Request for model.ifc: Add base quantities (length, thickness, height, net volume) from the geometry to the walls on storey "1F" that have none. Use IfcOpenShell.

First a look at what the model holds.

```python
import ifcopenshell
import ifcopenshell.util.element
import ifcopenshell.util.unit

model = ifcopenshell.open("model.ifc")
print(model.schema)
for unit_type in ("LENGTHUNIT", "AREAUNIT", "VOLUMEUNIT"):
    print(unit_type, ifcopenshell.util.unit.calculate_unit_scale(model, unit_type))
storey = next(s for s in model.by_type("IfcBuildingStorey") if s.Name == "1F")
walls = [e for e in ifcopenshell.util.element.get_decomposition(storey) if e.is_a("IfcWall")]
for e in sorted(walls, key=lambda e: e.id()):
    print(e.id(), e.is_a(), e.Name, list(ifcopenshell.util.element.get_psets(e, qtos_only=True)), sep=" | ")
```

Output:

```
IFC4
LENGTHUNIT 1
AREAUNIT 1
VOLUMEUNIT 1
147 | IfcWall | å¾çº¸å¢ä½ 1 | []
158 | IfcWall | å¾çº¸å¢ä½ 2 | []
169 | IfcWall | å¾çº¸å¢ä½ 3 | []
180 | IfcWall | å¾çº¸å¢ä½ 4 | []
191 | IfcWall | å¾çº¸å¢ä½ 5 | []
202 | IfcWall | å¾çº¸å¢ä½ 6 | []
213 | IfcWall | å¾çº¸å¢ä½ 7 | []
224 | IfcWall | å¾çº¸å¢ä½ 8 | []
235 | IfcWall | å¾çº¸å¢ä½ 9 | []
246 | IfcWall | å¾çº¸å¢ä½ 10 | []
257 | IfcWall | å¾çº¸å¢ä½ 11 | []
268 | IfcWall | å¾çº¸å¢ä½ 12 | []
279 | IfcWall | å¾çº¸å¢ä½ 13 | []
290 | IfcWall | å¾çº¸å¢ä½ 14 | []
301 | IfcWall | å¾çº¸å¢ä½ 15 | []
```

```python
import ifcopenshell
import ifcopenshell.api.pset
import ifcopenshell.geom
import ifcopenshell.util.element
import ifcopenshell.util.shape
import ifcopenshell.util.unit

model = ifcopenshell.open("model.ifc")
unit_scale = ifcopenshell.util.unit.calculate_unit_scale(model)
volume_scale = ifcopenshell.util.unit.calculate_unit_scale(model, "VOLUMEUNIT")
settings = ifcopenshell.geom.settings()

storey = next(s for s in model.by_type("IfcBuildingStorey") if s.Name == "1F")
walls = [e for e in ifcopenshell.util.element.get_decomposition(storey) if e.is_a("IfcWall")]

for e in sorted(walls, key=lambda e: e.id()):
    if ifcopenshell.util.element.get_psets(e, qtos_only=True, should_inherit=False):
        continue
    # Geometry comes back in metres, in the element's own axes.
    shape = ifcopenshell.geom.create_shape(settings, e)
    values = {
        "Length": ifcopenshell.util.shape.get_x(shape.geometry) / unit_scale,
        "Width": ifcopenshell.util.shape.get_y(shape.geometry) / unit_scale,
        "Height": ifcopenshell.util.shape.get_z(shape.geometry) / unit_scale,
        "NetVolume": ifcopenshell.util.shape.get_volume(shape.geometry) / volume_scale,
    }
    qto = ifcopenshell.api.pset.add_qto(model, product=e, name="Qto_WallBaseQuantities")
    ifcopenshell.api.pset.edit_qto(model, qto=qto, properties=values)
    print(e.id(), {k: round(v, 3) for k, v in values.items()})

model.write("model_updated.ifc")
```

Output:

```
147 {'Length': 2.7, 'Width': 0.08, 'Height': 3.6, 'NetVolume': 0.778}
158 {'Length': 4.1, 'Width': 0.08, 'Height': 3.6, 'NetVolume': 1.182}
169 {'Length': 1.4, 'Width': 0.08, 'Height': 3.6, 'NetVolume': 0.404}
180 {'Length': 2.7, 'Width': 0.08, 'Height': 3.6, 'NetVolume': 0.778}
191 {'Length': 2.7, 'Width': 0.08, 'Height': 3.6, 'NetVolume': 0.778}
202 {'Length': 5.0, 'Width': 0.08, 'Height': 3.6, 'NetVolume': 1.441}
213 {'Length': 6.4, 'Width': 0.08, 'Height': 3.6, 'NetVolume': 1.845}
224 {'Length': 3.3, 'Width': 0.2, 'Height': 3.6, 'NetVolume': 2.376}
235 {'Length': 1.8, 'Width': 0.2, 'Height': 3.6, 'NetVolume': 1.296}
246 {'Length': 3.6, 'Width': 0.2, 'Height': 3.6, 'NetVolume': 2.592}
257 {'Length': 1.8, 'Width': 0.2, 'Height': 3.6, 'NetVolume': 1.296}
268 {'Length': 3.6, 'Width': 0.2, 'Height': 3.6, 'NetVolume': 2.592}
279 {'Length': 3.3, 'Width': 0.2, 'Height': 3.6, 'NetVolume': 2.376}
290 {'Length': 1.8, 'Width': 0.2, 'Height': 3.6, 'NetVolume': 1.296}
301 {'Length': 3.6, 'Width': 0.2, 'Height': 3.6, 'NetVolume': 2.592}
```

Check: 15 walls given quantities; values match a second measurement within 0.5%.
